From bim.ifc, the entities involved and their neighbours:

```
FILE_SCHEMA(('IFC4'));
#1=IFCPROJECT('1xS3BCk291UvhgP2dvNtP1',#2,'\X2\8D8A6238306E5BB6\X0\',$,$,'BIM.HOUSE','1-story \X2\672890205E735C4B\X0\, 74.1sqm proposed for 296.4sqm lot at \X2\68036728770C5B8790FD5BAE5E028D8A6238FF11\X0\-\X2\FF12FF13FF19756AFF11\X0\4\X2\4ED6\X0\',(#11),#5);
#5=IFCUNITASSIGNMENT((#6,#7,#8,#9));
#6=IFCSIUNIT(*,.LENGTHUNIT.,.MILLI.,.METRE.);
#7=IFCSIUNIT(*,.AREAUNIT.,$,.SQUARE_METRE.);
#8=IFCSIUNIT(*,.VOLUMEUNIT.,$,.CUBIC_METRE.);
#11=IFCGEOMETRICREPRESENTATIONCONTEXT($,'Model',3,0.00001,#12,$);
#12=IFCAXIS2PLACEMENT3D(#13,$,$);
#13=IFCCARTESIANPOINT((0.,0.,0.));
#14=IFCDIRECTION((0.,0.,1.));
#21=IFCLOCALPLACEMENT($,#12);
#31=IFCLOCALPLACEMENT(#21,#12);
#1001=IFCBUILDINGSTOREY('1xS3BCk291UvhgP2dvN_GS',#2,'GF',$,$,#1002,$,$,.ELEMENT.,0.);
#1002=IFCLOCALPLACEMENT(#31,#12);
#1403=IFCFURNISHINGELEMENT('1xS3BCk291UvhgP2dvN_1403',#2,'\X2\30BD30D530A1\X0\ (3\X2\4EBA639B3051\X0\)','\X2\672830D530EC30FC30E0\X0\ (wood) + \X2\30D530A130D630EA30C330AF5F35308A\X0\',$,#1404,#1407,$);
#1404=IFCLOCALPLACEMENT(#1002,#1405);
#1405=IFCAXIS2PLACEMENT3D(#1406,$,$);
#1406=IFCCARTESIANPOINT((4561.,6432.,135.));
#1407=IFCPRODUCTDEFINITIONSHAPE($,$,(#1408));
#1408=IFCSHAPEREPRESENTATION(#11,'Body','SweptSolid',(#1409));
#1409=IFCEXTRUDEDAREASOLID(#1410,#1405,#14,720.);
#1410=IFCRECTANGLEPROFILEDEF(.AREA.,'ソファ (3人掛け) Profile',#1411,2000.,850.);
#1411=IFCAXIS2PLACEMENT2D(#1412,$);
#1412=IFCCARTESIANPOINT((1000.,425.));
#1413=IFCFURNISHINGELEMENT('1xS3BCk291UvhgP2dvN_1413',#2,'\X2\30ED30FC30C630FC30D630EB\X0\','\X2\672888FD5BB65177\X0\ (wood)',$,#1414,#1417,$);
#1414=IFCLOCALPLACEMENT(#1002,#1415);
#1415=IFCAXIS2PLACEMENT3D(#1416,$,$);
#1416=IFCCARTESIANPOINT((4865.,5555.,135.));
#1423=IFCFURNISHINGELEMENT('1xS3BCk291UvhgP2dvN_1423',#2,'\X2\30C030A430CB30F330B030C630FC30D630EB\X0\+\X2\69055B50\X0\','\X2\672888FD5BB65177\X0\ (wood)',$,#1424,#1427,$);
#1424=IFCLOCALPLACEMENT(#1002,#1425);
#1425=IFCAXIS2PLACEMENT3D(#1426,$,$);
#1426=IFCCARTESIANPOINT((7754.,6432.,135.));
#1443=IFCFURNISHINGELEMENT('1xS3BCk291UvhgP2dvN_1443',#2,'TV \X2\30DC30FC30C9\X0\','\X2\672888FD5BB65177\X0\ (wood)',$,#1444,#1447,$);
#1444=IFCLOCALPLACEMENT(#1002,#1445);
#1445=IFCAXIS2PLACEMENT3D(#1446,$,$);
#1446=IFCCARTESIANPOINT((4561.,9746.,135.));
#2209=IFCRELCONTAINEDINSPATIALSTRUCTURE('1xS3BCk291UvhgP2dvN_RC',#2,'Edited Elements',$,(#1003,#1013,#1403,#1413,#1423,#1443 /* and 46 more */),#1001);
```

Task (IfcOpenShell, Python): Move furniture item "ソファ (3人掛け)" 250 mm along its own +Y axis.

```python
import ifcopenshell
import ifcopenshell.api.geometry
import ifcopenshell.util.placement

model = ifcopenshell.open("bim.ifc")

item = model.by_id(1403)
matrix = ifcopenshell.util.placement.get_local_placement(item.ObjectPlacement)
matrix[:3, 3] += matrix[:3, 1] * 250.0
ifcopenshell.api.geometry.edit_object_placement(model, product=item, matrix=matrix, is_si=False)

print(ifcopenshell.util.placement.get_local_placement(item.ObjectPlacement).round(3) + 0.0)

model.write("bim-out.ifc")
```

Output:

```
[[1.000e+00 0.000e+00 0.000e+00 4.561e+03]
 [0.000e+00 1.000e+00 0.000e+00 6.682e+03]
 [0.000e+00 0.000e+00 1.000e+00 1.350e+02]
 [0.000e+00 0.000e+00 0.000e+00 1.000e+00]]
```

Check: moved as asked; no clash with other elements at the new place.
